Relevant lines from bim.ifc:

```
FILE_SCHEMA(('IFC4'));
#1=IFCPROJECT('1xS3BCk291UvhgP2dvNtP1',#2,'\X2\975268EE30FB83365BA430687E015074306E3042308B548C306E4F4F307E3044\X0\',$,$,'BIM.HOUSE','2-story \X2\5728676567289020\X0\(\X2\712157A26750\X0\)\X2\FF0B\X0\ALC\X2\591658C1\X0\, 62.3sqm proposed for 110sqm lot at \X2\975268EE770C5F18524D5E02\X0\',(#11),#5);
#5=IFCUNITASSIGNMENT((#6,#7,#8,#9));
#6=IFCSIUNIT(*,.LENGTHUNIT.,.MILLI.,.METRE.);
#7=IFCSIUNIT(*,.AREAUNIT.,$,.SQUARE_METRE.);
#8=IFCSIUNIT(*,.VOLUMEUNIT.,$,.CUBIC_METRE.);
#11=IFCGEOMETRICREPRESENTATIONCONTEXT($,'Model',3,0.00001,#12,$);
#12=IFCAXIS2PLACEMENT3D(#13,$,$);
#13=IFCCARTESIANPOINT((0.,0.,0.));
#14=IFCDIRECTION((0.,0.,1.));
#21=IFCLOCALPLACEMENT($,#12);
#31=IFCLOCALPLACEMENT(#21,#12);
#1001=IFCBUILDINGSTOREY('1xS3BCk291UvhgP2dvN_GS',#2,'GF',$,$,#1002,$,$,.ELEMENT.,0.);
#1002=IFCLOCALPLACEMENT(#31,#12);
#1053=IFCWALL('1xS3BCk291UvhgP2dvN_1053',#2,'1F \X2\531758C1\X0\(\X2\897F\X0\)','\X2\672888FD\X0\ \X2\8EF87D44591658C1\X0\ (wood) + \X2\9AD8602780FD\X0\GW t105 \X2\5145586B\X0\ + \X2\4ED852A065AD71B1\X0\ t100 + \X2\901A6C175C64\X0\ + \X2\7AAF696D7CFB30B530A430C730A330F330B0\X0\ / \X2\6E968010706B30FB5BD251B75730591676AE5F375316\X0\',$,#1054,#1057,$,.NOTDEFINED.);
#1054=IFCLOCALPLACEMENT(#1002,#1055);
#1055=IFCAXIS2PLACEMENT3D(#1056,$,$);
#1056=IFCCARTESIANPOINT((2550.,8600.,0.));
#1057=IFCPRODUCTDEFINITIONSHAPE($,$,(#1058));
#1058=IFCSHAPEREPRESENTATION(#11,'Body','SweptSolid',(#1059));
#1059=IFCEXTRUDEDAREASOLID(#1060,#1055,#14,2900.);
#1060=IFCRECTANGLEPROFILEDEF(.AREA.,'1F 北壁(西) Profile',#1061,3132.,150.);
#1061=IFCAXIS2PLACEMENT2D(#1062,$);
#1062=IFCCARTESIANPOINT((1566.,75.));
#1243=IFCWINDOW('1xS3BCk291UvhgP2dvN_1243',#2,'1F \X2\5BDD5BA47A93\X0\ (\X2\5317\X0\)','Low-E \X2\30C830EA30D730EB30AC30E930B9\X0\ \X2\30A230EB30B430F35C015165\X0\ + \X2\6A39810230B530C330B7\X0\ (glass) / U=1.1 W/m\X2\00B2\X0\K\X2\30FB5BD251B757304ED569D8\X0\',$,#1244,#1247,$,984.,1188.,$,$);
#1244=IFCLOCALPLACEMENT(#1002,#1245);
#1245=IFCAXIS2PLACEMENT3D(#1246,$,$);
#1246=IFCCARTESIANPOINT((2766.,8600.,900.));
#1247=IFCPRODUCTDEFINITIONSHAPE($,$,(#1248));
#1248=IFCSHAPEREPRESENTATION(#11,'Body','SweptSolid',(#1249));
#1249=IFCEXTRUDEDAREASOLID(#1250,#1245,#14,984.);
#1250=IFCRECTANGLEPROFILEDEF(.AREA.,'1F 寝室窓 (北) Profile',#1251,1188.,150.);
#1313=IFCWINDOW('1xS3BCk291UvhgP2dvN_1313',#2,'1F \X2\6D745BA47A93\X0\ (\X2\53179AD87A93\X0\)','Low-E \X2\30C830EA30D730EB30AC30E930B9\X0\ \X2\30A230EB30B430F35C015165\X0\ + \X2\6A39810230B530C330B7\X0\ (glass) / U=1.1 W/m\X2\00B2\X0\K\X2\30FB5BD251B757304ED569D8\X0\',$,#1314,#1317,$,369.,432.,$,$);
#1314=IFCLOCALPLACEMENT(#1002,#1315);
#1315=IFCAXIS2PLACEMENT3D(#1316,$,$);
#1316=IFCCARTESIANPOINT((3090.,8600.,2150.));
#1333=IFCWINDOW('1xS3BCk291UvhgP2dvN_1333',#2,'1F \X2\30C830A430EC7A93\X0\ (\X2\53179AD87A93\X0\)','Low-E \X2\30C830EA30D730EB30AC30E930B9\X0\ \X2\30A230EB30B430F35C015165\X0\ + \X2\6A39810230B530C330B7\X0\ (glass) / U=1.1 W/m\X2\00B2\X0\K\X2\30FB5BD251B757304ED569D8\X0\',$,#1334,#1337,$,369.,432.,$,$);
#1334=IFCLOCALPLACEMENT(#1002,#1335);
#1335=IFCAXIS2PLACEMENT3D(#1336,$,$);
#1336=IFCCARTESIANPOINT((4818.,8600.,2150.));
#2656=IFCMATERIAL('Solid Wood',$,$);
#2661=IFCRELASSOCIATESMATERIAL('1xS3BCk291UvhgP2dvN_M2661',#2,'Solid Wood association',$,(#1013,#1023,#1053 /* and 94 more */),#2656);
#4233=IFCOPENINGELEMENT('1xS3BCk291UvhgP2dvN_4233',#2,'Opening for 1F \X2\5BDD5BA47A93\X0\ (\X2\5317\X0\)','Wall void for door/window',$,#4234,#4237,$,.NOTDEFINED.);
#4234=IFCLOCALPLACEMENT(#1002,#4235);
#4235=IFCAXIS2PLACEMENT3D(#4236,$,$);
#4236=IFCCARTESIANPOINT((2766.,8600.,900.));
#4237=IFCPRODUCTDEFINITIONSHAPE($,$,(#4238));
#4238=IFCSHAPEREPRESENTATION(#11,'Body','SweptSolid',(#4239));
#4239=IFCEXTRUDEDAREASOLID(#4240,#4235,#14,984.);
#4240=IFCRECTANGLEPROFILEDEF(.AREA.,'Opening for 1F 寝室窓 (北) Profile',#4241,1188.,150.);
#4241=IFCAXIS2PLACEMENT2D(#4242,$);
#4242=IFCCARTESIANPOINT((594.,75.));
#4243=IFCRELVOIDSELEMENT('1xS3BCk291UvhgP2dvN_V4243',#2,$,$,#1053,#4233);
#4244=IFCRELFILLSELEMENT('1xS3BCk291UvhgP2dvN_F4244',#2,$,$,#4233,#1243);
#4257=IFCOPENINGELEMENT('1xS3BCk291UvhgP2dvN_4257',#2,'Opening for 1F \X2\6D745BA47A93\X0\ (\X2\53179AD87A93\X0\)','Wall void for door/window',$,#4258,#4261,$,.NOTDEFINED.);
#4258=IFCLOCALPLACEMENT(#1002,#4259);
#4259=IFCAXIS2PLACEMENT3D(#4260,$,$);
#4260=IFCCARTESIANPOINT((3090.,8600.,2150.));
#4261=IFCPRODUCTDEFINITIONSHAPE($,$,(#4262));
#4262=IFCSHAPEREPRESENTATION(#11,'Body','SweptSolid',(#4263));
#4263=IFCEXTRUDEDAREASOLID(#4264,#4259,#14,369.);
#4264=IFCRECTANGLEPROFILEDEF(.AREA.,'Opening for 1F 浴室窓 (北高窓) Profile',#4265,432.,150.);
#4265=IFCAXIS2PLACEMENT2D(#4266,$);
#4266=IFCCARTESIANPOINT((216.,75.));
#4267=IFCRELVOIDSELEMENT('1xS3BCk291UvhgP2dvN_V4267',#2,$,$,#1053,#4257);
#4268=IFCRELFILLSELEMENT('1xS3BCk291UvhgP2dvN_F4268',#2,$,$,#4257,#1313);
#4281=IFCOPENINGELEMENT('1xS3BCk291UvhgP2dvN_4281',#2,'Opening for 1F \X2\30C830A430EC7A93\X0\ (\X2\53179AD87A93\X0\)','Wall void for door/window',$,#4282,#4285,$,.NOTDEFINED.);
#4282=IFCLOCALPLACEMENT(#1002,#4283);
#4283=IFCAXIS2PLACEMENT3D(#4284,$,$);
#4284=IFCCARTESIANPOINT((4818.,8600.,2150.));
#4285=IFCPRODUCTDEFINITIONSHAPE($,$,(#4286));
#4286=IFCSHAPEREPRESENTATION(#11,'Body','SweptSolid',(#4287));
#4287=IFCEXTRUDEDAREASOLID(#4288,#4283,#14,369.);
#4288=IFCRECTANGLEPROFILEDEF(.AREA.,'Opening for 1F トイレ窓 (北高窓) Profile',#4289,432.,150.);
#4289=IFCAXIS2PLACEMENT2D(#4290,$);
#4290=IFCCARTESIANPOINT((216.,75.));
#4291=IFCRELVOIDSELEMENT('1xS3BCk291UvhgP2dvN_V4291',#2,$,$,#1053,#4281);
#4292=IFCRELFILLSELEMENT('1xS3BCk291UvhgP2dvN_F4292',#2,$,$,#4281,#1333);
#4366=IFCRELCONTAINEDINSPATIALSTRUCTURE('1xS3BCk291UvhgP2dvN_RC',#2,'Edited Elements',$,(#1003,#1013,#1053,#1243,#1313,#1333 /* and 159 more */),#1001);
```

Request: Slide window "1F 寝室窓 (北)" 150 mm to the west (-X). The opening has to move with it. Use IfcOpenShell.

```python
import ifcopenshell
import ifcopenshell.api.geometry
import ifcopenshell.util.placement
import ifcopenshell.util.unit

model = ifcopenshell.open("bim.ifc")
unit_scale = ifcopenshell.util.unit.calculate_unit_scale(model)

window = model.by_guid("1xS3BCk291UvhgP2dvN_1243")
opening = window.FillsVoids[0].RelatingOpeningElement
wall = opening.VoidsElements[0].RelatingBuildingElement

wall_matrix = ifcopenshell.util.placement.get_local_placement(wall.ObjectPlacement)
shift = wall_matrix[:3, 0] * -0.15 / unit_scale
before = ifcopenshell.util.placement.get_local_placement(window.ObjectPlacement)[:3, 3].copy()

# The window is not placed relative to its opening, so move both.
for product in (opening, window):
    matrix = ifcopenshell.util.placement.get_local_placement(product.ObjectPlacement)
    matrix[:3, 3] += shift
    ifcopenshell.api.geometry.edit_object_placement(model, product=product, matrix=matrix, is_si=False)

after = ifcopenshell.util.placement.get_local_placement(window.ObjectPlacement)[:3, 3]
print("window moved by", (after - before).round(3) + 0.0)

model.write("bim_rev.ifc")
```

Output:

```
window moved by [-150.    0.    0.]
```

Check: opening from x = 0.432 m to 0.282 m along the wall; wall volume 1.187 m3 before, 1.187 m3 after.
